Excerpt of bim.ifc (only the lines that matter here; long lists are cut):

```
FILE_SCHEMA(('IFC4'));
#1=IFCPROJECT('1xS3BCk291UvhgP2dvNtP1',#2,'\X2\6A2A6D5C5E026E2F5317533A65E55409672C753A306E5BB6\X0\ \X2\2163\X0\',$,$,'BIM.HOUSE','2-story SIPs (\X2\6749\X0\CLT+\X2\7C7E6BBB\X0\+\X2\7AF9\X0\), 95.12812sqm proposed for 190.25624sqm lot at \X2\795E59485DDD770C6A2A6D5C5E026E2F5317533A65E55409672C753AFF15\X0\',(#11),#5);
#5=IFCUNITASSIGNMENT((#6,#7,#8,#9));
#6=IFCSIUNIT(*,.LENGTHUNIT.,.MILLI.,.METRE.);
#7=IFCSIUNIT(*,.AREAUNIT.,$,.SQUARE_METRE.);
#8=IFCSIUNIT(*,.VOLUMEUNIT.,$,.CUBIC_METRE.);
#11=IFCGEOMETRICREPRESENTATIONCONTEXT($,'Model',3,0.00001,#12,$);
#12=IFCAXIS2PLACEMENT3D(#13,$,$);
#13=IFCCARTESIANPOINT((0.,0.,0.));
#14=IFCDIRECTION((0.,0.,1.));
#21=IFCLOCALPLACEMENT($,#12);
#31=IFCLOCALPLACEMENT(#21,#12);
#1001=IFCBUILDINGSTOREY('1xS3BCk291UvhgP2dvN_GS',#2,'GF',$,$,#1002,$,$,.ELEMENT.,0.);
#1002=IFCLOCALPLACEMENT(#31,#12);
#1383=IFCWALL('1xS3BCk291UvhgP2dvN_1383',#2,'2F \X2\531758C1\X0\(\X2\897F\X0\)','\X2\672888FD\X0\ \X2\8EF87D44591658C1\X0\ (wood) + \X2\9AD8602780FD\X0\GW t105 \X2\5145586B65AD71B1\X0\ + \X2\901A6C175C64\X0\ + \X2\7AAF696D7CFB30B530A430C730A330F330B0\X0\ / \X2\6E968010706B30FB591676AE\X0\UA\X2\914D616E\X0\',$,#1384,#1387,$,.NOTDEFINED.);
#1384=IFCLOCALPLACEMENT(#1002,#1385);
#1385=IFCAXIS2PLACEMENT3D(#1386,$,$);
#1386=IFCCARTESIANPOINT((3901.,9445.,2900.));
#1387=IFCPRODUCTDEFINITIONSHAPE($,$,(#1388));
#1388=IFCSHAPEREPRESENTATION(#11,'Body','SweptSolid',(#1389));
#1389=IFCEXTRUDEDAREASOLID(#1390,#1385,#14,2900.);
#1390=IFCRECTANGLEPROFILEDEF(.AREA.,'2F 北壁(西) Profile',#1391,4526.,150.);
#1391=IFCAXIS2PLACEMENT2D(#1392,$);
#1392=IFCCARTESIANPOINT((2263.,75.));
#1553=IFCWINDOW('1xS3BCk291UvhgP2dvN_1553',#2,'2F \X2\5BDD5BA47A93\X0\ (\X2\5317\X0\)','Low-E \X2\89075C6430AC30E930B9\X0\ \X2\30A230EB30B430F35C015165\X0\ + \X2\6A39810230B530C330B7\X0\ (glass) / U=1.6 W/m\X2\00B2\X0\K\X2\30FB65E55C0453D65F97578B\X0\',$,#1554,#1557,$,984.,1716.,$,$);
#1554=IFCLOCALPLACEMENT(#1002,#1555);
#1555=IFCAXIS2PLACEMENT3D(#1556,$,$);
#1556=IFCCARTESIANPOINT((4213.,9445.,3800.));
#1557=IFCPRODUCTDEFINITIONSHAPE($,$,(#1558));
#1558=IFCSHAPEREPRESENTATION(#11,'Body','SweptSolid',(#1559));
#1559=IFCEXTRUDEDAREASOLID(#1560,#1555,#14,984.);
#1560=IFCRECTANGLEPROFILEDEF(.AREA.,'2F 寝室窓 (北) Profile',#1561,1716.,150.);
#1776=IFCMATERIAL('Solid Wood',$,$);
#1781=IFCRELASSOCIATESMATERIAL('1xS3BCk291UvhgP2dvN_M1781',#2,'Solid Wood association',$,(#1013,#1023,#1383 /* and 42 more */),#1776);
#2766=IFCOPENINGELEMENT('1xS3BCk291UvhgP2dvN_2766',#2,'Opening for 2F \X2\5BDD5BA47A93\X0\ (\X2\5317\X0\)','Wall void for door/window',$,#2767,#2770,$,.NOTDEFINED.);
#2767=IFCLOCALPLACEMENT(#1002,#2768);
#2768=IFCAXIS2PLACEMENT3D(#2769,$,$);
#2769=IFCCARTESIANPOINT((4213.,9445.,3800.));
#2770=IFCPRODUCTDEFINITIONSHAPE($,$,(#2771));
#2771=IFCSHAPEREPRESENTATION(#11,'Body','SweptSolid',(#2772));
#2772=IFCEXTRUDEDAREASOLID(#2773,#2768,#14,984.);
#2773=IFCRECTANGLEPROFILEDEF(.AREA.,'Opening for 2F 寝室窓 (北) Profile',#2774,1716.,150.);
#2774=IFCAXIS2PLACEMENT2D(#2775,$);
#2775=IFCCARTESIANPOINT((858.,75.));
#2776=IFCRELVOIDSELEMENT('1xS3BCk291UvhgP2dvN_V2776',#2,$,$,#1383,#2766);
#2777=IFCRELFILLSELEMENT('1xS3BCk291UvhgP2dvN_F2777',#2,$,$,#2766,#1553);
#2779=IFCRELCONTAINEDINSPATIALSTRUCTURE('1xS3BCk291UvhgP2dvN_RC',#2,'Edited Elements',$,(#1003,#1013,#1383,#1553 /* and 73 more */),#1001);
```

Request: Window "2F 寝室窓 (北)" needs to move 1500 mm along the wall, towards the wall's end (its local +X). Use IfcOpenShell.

```python
import ifcopenshell
import ifcopenshell.api.geometry
import ifcopenshell.util.placement
import ifcopenshell.util.unit

model = ifcopenshell.open("bim.ifc")
unit_scale = ifcopenshell.util.unit.calculate_unit_scale(model)

window = model.by_guid("1xS3BCk291UvhgP2dvN_1553")
opening = window.FillsVoids[0].RelatingOpeningElement
wall = opening.VoidsElements[0].RelatingBuildingElement

wall_matrix = ifcopenshell.util.placement.get_local_placement(wall.ObjectPlacement)
shift = wall_matrix[:3, 0] * 1.5 / unit_scale
before = ifcopenshell.util.placement.get_local_placement(window.ObjectPlacement)[:3, 3].copy()

# The window is not placed relative to its opening, so move both.
for product in (opening, window):
    matrix = ifcopenshell.util.placement.get_local_placement(product.ObjectPlacement)
    matrix[:3, 3] += shift
    ifcopenshell.api.geometry.edit_object_placement(model, product=product, matrix=matrix, is_si=False)

after = ifcopenshell.util.placement.get_local_placement(window.ObjectPlacement)[:3, 3]
print("window moved by", (after - before).round(3) + 0.0)

model.write("bim_updated.ifc")
```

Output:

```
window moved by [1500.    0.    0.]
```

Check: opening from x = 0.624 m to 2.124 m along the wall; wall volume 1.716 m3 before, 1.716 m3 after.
